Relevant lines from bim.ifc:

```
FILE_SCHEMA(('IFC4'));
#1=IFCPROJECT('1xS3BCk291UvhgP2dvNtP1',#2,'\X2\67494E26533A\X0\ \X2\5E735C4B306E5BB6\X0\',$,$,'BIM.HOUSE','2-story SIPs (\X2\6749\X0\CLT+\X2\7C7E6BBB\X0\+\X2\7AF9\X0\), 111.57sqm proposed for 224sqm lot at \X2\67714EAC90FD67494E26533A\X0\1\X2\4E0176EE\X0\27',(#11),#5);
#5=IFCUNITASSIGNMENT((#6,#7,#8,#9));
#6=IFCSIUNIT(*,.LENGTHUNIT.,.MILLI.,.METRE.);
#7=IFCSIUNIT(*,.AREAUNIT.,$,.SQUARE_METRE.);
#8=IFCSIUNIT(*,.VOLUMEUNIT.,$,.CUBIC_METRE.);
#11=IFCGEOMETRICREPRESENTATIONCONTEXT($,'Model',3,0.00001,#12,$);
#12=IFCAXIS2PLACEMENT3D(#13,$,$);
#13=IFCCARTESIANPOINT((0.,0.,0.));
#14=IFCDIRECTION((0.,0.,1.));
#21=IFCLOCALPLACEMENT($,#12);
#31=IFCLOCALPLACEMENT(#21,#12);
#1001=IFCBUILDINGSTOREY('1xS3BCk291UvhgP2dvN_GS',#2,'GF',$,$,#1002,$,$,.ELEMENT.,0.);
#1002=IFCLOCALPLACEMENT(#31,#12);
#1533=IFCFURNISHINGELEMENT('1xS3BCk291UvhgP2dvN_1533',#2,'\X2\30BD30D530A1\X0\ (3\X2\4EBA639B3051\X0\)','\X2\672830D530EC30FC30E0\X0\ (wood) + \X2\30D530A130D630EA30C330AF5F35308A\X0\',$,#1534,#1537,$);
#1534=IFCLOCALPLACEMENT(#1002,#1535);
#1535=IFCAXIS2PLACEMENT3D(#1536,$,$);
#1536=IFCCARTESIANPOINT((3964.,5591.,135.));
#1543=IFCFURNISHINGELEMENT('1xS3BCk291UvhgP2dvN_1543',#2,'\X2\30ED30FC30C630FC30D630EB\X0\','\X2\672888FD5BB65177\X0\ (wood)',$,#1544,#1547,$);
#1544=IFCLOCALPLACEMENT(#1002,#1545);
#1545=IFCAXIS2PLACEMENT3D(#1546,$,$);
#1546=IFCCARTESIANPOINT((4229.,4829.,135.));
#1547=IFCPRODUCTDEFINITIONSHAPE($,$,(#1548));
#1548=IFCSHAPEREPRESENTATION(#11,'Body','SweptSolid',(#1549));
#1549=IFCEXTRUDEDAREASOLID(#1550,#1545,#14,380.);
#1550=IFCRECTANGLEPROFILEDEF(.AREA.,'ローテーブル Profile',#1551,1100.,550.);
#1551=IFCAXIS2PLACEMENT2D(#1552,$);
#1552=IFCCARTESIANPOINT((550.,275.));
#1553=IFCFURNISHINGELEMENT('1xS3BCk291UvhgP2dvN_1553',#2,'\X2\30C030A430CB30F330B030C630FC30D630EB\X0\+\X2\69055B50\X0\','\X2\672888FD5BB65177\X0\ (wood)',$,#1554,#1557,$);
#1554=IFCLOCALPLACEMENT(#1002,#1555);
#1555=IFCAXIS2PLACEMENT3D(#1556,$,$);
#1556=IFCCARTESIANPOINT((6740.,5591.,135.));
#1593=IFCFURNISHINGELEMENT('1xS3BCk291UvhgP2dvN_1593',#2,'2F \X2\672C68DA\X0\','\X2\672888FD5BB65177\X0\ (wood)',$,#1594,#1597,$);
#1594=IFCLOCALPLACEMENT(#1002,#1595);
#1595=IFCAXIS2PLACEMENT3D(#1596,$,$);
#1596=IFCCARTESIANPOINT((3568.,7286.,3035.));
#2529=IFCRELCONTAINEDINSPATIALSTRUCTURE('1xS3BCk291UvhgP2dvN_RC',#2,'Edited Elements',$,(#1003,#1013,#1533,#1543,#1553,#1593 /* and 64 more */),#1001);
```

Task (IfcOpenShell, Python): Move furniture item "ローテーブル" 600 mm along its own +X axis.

```python
import ifcopenshell
import ifcopenshell.api.geometry
import ifcopenshell.util.placement

model = ifcopenshell.open("bim.ifc")

item = model.by_guid("1xS3BCk291UvhgP2dvN_1543")
matrix = ifcopenshell.util.placement.get_local_placement(item.ObjectPlacement)
matrix[:3, 3] += matrix[:3, 0] * 600.0
ifcopenshell.api.geometry.edit_object_placement(model, product=item, matrix=matrix, is_si=False)

print(ifcopenshell.util.placement.get_local_placement(item.ObjectPlacement).round(3) + 0.0)

model.write("bim-out.ifc")
```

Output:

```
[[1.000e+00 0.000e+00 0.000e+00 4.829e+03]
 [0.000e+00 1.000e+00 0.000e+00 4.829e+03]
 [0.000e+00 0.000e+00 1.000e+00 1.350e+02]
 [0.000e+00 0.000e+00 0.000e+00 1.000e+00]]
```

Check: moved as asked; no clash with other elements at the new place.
